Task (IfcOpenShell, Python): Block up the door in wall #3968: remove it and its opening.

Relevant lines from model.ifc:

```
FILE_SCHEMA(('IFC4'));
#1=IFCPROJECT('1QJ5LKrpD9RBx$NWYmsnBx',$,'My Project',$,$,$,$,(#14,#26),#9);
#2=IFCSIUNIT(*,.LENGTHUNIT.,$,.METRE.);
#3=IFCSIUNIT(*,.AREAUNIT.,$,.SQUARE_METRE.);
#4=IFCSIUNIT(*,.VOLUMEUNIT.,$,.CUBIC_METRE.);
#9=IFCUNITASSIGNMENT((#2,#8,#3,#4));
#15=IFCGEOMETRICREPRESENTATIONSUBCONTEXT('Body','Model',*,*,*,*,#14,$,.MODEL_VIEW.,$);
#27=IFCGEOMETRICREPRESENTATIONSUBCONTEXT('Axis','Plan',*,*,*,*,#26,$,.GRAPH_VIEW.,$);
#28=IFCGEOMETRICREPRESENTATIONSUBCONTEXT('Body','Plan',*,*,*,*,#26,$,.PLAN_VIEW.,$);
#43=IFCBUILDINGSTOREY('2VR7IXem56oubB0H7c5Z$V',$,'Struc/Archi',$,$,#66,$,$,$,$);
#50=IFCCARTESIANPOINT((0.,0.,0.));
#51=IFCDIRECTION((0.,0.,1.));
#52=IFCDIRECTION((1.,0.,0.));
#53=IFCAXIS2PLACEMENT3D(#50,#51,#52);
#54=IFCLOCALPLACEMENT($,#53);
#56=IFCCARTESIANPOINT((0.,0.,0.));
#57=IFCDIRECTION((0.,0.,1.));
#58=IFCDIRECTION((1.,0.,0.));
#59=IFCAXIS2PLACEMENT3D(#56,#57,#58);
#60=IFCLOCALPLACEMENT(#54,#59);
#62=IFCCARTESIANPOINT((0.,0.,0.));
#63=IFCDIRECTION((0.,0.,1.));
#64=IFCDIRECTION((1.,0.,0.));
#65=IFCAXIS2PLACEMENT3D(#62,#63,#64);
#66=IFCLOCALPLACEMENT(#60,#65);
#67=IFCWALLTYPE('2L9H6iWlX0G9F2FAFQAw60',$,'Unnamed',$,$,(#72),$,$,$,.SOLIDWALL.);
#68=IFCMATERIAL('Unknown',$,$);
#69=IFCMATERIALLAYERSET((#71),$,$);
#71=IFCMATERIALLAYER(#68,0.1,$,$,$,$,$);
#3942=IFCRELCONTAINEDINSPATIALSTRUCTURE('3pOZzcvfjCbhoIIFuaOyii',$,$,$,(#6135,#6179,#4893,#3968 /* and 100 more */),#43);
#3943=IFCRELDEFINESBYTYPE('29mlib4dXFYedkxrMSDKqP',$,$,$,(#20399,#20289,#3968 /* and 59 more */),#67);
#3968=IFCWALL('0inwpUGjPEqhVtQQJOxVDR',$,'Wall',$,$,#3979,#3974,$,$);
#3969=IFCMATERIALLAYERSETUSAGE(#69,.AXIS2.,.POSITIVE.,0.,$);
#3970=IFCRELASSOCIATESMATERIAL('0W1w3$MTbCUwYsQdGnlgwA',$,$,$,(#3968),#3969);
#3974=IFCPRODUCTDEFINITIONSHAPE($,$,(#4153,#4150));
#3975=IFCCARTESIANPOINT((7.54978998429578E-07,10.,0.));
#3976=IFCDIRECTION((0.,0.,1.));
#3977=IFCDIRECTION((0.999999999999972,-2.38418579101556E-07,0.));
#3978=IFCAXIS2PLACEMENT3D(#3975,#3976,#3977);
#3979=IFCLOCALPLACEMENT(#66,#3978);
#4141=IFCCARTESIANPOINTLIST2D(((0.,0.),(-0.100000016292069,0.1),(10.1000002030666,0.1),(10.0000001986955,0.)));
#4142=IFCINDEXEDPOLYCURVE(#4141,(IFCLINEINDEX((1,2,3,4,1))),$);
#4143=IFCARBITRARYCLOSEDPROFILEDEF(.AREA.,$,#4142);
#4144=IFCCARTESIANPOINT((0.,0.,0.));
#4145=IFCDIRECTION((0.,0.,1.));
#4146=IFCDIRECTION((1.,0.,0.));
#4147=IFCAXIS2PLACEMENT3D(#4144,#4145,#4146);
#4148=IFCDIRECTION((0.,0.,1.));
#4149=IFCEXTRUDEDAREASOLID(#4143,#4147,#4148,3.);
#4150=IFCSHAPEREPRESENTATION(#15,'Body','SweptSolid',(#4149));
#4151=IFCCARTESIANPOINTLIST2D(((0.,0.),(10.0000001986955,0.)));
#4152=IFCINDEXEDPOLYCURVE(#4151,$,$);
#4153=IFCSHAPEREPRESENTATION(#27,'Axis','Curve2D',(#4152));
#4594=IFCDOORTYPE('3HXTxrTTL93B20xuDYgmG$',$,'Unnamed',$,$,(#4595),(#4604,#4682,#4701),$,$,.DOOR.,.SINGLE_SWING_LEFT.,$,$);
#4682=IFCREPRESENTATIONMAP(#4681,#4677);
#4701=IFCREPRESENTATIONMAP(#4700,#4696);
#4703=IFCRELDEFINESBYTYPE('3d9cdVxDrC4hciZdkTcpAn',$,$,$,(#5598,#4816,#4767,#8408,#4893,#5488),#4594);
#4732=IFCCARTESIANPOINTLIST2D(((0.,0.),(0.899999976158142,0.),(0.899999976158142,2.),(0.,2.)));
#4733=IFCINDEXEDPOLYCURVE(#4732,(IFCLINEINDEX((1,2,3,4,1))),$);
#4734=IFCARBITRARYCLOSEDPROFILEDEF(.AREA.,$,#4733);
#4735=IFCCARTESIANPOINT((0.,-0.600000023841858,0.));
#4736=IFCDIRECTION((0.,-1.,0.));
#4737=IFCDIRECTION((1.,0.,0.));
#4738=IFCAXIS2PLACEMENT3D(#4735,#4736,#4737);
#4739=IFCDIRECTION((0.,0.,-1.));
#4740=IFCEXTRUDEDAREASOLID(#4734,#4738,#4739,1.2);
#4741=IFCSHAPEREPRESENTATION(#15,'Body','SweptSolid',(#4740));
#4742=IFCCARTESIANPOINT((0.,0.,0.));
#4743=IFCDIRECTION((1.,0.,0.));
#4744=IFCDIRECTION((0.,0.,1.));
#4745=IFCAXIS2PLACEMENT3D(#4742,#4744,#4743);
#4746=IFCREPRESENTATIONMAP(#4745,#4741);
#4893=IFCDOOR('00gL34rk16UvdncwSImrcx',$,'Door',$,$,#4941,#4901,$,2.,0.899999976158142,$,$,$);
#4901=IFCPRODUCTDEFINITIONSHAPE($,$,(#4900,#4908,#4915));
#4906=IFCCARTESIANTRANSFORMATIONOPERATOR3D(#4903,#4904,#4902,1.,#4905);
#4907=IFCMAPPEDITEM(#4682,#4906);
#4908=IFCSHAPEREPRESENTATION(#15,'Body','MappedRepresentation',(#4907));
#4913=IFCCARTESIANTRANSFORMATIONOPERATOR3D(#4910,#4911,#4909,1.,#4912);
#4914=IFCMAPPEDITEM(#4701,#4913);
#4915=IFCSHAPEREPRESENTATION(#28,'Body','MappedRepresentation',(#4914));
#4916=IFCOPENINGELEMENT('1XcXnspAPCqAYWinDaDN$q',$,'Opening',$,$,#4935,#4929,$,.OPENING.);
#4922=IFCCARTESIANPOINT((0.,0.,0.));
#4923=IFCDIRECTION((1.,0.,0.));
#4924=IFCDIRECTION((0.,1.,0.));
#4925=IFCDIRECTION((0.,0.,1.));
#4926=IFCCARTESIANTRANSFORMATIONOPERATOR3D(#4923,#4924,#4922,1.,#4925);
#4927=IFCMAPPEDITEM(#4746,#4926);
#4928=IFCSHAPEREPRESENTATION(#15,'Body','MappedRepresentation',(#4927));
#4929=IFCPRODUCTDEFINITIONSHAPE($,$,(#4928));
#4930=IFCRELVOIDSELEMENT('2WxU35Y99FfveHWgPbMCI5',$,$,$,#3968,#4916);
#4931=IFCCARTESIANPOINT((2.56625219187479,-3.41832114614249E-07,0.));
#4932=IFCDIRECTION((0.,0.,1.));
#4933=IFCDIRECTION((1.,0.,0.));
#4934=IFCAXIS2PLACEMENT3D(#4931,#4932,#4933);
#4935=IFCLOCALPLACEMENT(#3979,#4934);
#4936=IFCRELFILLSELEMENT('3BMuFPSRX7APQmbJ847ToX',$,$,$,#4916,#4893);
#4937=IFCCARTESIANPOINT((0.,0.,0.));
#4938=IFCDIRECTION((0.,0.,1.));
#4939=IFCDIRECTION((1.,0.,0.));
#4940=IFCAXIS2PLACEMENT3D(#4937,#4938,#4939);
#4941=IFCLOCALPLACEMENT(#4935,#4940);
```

```python
import ifcopenshell
import ifcopenshell.api.feature
import ifcopenshell.api.root
import ifcopenshell.geom
import ifcopenshell.util.shape

model = ifcopenshell.open("model.ifc")
settings = ifcopenshell.geom.settings()


def volume(element):
    """Net volume in cubic metres, openings subtracted."""
    shape = ifcopenshell.geom.create_shape(settings, element)
    return ifcopenshell.util.shape.get_volume(shape.geometry)


door = model.by_guid("00gL34rk16UvdncwSImrcx")
opening = door.FillsVoids[0].RelatingOpeningElement
wall = opening.VoidsElements[0].RelatingBuildingElement
before = volume(wall)

ifcopenshell.api.root.remove_product(model, product=door)
ifcopenshell.api.feature.remove_feature(model, feature=opening)

after = volume(wall)

print(f"wall volume {before:.3f} -> {after:.3f} m3")

model.write("model_rev.ifc")
```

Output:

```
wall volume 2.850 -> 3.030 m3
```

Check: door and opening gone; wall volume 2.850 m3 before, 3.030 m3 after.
